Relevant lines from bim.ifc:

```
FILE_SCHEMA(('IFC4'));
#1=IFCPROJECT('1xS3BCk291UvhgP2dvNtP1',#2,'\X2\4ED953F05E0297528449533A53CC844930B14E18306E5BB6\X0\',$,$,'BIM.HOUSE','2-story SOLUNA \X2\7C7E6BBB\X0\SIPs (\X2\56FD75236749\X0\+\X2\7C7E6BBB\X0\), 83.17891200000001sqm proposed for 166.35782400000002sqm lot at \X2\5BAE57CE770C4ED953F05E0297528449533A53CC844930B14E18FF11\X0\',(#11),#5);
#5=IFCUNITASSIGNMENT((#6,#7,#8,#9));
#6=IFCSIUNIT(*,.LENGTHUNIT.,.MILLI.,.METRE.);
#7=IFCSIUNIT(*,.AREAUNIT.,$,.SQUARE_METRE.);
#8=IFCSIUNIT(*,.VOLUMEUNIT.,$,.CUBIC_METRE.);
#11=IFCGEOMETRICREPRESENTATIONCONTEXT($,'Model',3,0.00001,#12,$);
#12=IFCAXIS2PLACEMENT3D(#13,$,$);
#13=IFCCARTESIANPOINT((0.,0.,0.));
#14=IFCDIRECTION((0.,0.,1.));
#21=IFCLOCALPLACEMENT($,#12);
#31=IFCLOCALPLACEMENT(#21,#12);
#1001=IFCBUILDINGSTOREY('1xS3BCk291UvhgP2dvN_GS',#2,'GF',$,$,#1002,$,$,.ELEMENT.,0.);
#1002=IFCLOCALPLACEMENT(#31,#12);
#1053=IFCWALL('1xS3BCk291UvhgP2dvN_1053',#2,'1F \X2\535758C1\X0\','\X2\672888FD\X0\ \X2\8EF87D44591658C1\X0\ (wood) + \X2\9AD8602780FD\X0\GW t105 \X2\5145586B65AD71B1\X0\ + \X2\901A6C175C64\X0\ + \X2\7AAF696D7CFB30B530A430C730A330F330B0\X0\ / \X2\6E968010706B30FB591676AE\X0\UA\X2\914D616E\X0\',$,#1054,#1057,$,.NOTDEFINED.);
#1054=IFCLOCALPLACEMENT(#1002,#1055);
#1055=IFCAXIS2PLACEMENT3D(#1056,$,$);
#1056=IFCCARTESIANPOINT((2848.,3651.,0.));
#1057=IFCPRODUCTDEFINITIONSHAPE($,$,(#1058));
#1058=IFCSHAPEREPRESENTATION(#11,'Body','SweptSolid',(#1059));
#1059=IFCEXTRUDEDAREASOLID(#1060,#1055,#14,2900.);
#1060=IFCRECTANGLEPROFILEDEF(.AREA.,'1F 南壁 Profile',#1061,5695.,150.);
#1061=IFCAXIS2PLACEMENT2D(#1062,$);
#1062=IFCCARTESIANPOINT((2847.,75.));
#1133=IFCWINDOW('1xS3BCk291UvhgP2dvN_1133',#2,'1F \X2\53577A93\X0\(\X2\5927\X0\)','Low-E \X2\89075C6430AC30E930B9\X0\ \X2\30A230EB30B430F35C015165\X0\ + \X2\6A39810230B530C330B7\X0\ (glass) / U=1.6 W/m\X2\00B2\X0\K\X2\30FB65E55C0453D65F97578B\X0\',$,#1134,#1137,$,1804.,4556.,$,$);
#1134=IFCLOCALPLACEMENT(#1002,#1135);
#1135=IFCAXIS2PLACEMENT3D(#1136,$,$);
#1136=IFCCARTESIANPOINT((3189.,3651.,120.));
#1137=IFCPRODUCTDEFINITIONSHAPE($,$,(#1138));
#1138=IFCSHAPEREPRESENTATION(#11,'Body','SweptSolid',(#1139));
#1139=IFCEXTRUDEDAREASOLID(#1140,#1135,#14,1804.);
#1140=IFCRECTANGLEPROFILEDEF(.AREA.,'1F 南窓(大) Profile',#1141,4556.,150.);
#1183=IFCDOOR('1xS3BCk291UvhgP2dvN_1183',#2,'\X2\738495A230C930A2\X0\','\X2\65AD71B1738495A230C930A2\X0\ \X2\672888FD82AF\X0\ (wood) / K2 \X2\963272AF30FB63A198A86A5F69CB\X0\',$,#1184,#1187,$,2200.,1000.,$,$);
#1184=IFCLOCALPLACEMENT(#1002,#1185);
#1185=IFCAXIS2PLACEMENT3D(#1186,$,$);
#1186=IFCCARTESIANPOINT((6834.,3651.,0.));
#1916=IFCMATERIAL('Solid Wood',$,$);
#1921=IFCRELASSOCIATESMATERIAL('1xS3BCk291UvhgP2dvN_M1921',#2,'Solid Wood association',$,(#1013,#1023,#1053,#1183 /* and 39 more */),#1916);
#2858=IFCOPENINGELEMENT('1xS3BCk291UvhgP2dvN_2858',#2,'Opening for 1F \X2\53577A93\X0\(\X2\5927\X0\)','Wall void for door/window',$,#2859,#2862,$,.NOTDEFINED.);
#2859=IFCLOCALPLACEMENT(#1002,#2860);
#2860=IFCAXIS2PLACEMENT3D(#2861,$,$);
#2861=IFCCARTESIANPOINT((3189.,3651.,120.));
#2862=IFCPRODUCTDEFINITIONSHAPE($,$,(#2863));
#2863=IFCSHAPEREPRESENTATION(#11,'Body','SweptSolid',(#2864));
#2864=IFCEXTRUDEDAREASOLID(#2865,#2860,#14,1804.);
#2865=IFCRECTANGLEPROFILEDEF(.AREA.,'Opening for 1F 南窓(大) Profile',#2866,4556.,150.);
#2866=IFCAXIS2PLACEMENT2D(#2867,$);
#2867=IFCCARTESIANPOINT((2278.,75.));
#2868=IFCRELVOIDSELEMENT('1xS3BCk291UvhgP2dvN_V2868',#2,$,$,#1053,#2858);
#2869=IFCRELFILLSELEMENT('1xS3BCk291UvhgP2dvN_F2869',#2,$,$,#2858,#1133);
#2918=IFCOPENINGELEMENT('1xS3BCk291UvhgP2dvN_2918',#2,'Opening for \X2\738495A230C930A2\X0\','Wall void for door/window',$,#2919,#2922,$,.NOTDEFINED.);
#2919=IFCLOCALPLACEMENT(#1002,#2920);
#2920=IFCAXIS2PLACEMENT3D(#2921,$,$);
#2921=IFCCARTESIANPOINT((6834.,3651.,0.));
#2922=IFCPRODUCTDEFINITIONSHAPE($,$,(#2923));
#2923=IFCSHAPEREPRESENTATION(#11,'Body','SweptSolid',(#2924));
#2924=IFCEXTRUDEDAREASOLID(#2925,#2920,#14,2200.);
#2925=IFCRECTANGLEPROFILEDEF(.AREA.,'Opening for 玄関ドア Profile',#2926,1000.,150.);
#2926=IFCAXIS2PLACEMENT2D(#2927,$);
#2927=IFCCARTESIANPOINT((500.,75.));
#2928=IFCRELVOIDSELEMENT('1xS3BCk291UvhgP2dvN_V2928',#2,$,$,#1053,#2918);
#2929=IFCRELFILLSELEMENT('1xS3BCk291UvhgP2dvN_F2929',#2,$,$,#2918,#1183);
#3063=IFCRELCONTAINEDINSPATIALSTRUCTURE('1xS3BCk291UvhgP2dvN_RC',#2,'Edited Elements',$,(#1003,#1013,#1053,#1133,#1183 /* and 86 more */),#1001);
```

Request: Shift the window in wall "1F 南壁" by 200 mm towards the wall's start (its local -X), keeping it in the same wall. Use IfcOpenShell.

```python
import ifcopenshell
import ifcopenshell.api.geometry
import ifcopenshell.util.placement

model = ifcopenshell.open("bim.ifc")

window = model.by_guid("1xS3BCk291UvhgP2dvN_1133")
opening = window.FillsVoids[0].RelatingOpeningElement
wall = opening.VoidsElements[0].RelatingBuildingElement

wall_matrix = ifcopenshell.util.placement.get_local_placement(wall.ObjectPlacement)
shift = wall_matrix[:3, 0] * -200.0
before = ifcopenshell.util.placement.get_local_placement(window.ObjectPlacement)[:3, 3].copy()

# The window is not placed relative to its opening, so move both.
for product in (opening, window):
    matrix = ifcopenshell.util.placement.get_local_placement(product.ObjectPlacement)
    matrix[:3, 3] += shift
    ifcopenshell.api.geometry.edit_object_placement(model, product=product, matrix=matrix, is_si=False)

after = ifcopenshell.util.placement.get_local_placement(window.ObjectPlacement)[:3, 3]
print("window moved by", (after - before).round(3) + 0.0)

model.write("bim_v2.ifc")
```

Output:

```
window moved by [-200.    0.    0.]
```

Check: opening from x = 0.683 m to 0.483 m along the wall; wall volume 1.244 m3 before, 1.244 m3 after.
